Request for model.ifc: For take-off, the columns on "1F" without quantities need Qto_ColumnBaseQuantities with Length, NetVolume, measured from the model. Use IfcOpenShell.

First a look at what the model holds.

```python
import ifcopenshell
import ifcopenshell.util.element
import ifcopenshell.util.unit

model = ifcopenshell.open("model.ifc")
print(model.schema)
for unit_type in ("LENGTHUNIT", "AREAUNIT", "VOLUMEUNIT"):
    print(unit_type, ifcopenshell.util.unit.calculate_unit_scale(model, unit_type))
storey = next(s for s in model.by_type("IfcBuildingStorey") if s.Name == "1F")
columns = [e for e in ifcopenshell.util.element.get_decomposition(storey) if e.is_a("IfcColumn")]
for e in sorted(columns, key=lambda e: e.id()):
    print(e.id(), e.is_a(), e.Name, list(ifcopenshell.util.element.get_psets(e, qtos_only=True)), sep=" | ")
```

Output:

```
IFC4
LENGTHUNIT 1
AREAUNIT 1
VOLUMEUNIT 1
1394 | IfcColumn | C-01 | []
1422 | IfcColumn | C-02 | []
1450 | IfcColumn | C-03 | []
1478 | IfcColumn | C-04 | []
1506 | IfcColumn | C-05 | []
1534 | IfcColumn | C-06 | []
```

```python
import ifcopenshell
import ifcopenshell.api.pset
import ifcopenshell.geom
import ifcopenshell.util.element
import ifcopenshell.util.shape
import ifcopenshell.util.unit

model = ifcopenshell.open("model.ifc")
unit_scale = ifcopenshell.util.unit.calculate_unit_scale(model)
volume_scale = ifcopenshell.util.unit.calculate_unit_scale(model, "VOLUMEUNIT")
settings = ifcopenshell.geom.settings()

storey = next(s for s in model.by_type("IfcBuildingStorey") if s.Name == "1F")
columns = [e for e in ifcopenshell.util.element.get_decomposition(storey) if e.is_a("IfcColumn")]

for e in sorted(columns, key=lambda e: e.id()):
    if ifcopenshell.util.element.get_psets(e, qtos_only=True, should_inherit=False):
        continue
    # Geometry comes back in metres, in the element's own axes.
    shape = ifcopenshell.geom.create_shape(settings, e)
    values = {
        "Length": ifcopenshell.util.shape.get_z(shape.geometry) / unit_scale,
        "NetVolume": ifcopenshell.util.shape.get_volume(shape.geometry) / volume_scale,
    }
    qto = ifcopenshell.api.pset.add_qto(model, product=e, name="Qto_ColumnBaseQuantities")
    ifcopenshell.api.pset.edit_qto(model, qto=qto, properties=values)
    print(e.id(), {k: round(v, 3) for k, v in values.items()})

model.write("model_rev.ifc")
```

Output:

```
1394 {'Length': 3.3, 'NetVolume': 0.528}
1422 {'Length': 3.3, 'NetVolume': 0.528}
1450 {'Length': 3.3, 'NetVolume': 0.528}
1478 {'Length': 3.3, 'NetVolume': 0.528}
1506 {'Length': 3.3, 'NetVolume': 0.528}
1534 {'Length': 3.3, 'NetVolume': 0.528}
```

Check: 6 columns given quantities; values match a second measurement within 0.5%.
